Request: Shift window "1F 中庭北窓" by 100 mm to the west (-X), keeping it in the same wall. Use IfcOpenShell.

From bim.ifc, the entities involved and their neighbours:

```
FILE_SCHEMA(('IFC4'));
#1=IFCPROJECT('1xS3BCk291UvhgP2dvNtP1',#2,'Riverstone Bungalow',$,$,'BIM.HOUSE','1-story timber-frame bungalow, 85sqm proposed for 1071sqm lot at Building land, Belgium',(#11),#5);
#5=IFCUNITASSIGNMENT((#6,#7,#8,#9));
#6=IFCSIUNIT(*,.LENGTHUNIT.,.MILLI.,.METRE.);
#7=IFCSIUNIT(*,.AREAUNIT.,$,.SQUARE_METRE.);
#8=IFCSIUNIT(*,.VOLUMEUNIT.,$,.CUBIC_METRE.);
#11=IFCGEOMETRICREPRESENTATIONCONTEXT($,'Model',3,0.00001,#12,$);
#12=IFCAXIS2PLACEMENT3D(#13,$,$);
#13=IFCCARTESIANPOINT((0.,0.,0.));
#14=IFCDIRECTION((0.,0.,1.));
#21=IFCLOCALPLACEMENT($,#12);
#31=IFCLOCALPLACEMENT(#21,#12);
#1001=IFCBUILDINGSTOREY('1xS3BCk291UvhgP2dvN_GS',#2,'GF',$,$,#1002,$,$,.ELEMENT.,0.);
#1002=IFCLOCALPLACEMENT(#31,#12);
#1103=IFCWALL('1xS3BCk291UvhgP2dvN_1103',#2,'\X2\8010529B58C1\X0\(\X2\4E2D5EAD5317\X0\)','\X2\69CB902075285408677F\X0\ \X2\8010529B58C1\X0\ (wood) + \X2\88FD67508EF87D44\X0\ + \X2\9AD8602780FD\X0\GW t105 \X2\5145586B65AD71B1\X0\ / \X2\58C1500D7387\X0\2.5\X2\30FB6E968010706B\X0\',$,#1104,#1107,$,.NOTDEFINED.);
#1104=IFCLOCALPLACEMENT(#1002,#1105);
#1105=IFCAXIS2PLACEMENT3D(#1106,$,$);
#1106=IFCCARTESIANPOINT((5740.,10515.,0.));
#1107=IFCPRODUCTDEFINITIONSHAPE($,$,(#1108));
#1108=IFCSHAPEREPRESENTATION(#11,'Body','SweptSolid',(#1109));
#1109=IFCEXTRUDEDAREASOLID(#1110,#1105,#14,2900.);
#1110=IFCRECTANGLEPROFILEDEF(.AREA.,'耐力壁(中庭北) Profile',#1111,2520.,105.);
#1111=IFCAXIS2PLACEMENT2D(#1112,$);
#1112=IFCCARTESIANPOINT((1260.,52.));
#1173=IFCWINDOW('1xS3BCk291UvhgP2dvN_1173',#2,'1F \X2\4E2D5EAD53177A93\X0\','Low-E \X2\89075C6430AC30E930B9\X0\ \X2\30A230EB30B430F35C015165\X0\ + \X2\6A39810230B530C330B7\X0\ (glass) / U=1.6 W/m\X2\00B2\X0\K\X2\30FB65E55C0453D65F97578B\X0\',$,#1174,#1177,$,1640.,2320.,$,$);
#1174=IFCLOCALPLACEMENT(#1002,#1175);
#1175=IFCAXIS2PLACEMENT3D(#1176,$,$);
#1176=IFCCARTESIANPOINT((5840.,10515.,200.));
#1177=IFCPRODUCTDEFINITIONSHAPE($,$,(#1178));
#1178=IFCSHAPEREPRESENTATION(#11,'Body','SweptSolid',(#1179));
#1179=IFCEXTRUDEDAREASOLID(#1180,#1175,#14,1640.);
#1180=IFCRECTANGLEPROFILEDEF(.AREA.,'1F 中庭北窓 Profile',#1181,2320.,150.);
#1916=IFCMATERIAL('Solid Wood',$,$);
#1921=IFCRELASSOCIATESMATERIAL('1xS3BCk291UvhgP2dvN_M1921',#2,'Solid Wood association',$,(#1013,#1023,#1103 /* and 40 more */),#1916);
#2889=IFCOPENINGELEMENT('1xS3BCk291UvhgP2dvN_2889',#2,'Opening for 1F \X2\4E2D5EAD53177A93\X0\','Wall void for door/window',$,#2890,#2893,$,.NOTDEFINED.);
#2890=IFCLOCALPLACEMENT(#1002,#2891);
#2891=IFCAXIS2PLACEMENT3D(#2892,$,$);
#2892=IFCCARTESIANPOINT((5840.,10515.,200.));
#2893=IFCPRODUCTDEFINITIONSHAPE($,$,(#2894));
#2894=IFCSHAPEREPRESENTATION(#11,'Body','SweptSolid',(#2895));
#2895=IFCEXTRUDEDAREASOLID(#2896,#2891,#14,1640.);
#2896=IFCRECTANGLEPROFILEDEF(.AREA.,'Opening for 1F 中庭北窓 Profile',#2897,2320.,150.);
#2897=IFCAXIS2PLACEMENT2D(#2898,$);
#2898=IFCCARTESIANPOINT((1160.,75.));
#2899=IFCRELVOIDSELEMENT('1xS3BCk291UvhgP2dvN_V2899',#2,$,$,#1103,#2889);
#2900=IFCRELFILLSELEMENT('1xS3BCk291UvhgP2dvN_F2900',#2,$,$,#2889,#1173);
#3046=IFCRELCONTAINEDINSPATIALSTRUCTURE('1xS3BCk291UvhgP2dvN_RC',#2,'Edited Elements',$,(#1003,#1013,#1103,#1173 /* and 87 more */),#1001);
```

```python
import ifcopenshell
import ifcopenshell.api.geometry
import ifcopenshell.util.placement

model = ifcopenshell.open("bim.ifc")

window = model.by_guid("1xS3BCk291UvhgP2dvN_1173")
opening = window.FillsVoids[0].RelatingOpeningElement
wall = opening.VoidsElements[0].RelatingBuildingElement

wall_matrix = ifcopenshell.util.placement.get_local_placement(wall.ObjectPlacement)
shift = wall_matrix[:3, 0] * -100.0
before = ifcopenshell.util.placement.get_local_placement(window.ObjectPlacement)[:3, 3].copy()

# The window is not placed relative to its opening, so move both.
for product in (opening, window):
    matrix = ifcopenshell.util.placement.get_local_placement(product.ObjectPlacement)
    matrix[:3, 3] += shift
    ifcopenshell.api.geometry.edit_object_placement(model, product=product, matrix=matrix, is_si=False)

after = ifcopenshell.util.placement.get_local_placement(window.ObjectPlacement)[:3, 3]
print("window moved by", (after - before).round(3) + 0.0)

model.write("bim_edited.ifc")
```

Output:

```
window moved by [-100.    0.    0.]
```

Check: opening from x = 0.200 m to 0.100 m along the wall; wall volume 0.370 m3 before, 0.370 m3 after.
